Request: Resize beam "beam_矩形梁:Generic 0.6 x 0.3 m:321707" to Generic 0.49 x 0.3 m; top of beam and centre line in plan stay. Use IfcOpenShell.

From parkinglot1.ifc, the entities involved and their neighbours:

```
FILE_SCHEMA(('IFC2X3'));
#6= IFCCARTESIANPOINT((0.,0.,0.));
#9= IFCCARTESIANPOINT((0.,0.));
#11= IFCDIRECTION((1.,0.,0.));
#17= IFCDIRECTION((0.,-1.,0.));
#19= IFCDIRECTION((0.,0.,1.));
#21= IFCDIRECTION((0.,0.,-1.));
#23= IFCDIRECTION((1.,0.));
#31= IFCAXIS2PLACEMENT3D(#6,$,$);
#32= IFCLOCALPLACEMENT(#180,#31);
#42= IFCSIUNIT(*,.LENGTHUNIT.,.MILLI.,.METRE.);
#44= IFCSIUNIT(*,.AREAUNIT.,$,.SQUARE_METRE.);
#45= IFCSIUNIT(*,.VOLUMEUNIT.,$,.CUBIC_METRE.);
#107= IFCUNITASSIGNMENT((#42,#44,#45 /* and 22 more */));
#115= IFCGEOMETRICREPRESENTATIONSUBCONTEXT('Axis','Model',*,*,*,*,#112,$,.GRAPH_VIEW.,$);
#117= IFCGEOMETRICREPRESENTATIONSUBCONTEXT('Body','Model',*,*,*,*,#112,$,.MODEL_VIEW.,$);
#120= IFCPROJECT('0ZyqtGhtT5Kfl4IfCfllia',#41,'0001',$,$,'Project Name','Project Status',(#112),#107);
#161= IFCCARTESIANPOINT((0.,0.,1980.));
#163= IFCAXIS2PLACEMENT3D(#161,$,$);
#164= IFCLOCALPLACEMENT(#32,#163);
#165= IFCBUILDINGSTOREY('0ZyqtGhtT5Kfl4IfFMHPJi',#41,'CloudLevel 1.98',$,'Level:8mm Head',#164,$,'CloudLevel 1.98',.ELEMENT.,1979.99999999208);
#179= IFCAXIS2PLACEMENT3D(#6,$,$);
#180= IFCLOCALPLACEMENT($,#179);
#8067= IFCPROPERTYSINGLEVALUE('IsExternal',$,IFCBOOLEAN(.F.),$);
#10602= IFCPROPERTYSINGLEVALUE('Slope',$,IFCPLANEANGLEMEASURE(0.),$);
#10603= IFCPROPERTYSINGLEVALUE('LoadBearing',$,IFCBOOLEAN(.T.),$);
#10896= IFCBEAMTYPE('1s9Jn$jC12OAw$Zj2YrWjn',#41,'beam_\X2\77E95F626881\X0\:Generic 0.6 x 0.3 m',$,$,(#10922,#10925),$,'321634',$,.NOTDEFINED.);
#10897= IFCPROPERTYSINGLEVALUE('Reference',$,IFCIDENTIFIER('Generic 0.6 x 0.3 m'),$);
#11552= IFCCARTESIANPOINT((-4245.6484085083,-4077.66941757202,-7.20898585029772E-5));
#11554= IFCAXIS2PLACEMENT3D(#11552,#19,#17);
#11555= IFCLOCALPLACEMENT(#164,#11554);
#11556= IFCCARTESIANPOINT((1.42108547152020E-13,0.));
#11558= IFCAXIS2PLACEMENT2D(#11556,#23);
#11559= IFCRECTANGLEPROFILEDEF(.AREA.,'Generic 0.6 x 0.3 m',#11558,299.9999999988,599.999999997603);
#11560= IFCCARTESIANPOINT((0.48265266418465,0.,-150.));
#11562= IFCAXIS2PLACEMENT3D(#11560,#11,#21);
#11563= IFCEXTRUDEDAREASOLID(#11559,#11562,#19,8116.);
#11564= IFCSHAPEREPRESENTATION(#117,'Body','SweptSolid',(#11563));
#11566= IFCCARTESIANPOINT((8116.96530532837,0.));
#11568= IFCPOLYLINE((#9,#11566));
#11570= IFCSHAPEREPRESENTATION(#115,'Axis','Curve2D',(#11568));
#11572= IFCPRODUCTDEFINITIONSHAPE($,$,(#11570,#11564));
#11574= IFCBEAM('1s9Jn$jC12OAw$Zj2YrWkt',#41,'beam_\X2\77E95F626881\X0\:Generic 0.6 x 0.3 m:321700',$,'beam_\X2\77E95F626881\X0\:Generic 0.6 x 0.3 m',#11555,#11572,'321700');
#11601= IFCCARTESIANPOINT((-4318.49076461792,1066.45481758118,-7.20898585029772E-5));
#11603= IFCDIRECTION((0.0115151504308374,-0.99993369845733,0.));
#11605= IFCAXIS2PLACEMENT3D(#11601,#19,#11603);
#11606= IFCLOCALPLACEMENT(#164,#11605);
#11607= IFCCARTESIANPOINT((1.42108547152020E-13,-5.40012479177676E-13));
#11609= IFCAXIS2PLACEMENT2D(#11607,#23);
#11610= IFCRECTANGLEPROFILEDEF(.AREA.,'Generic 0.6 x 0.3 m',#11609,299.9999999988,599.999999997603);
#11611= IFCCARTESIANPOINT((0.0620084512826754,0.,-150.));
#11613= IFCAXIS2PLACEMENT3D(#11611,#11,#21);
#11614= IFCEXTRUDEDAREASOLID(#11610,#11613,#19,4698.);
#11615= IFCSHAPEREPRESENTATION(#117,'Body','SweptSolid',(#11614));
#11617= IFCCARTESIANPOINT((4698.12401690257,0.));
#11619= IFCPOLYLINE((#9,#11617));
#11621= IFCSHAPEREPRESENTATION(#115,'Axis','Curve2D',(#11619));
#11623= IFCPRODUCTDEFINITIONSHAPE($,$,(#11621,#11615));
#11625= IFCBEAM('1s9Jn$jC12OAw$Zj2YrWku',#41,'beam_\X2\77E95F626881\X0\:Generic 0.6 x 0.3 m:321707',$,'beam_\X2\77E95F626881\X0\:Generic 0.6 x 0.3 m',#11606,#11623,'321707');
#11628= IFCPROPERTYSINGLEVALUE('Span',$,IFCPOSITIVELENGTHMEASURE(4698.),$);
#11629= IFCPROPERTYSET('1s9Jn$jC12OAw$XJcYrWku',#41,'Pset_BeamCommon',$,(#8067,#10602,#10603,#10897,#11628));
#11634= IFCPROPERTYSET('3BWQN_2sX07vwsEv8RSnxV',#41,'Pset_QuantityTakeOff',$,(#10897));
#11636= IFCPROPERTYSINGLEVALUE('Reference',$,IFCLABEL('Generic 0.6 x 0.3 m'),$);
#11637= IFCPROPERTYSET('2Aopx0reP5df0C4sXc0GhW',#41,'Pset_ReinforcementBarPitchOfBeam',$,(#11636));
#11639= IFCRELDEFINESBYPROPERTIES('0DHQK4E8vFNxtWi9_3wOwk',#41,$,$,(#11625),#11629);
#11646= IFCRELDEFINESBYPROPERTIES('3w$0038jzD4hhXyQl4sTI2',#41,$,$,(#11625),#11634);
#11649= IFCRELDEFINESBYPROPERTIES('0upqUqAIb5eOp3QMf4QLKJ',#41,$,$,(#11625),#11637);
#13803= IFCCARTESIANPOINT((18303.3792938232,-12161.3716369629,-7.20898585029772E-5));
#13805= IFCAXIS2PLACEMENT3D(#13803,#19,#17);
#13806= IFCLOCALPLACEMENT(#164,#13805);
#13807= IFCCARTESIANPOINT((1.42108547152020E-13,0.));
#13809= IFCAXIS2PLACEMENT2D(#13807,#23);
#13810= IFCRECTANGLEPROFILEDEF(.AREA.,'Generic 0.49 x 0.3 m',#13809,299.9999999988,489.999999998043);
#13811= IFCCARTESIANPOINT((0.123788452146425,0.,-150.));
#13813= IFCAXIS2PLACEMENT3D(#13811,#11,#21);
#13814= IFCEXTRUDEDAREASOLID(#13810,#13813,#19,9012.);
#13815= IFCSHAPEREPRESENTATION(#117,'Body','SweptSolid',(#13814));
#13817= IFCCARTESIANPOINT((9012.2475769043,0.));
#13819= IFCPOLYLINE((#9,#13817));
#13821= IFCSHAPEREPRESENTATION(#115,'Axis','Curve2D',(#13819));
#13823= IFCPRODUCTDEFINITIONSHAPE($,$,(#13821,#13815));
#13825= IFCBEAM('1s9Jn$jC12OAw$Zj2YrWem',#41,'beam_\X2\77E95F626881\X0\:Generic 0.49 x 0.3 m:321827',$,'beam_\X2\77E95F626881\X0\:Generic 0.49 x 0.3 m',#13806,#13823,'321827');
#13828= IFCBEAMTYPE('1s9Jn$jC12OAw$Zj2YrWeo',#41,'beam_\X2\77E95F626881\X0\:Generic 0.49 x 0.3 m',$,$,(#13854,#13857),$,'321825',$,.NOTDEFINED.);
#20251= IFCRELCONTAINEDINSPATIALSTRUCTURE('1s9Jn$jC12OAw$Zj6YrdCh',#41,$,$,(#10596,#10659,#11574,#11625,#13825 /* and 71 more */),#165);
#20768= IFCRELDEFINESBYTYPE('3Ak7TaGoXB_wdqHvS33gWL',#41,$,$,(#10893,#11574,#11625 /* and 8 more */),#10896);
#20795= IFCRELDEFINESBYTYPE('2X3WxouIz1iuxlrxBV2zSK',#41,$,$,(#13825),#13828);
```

```python
import ifcopenshell
import ifcopenshell.api.pset
import ifcopenshell.api.type
import ifcopenshell.util.element
import ifcopenshell.util.representation

model = ifcopenshell.open("parkinglot1.ifc")

member = model.by_guid("1s9Jn$jC12OAw$Zj2YrWku")
source = next(p for p in model.by_type("IfcRectangleProfileDef") if p.ProfileName == "Generic 0.49 x 0.3 m")

body = ifcopenshell.util.representation.get_representation(member, "Model", "Body")
solid = body.Items[0]
old_profile = solid.SweptArea

# Copy the section's sizes but keep this member's own profile position.
profile = ifcopenshell.util.element.copy(model, source)
# Profiles are centred, so shift by half the change in depth to hold the top.
shift = (old_profile.XDim - profile.XDim) / 2
x, y = old_profile.Position.Location.Coordinates
up = (-1.0, 0.0)  # upwards, in the solid's own plane
location = model.createIfcCartesianPoint((x + up[0] * shift, y + up[1] * shift))
profile.Position = model.createIfcAxis2Placement2D(location, old_profile.Position.RefDirection)
solid.SweptArea = profile
if not model.get_total_inverses(old_profile):
    ifcopenshell.util.element.remove_deep2(model, old_profile)

new_type = model.by_guid("1s9Jn$jC12OAw$Zj2YrWeo")
ifcopenshell.api.type.assign_type(
    model, related_objects=[member], relating_type=new_type, should_map_representations=False
)
member.Name = member.Name.replace("Generic 0.6 x 0.3 m", "Generic 0.49 x 0.3 m")
member.ObjectType = "beam_矩形梁:Generic 0.49 x 0.3 m"
pset = model.by_id(ifcopenshell.util.element.get_pset(member, "Pset_BeamCommon", should_inherit=False)["id"])
ifcopenshell.api.pset.edit_pset(model, pset=pset, properties={"Reference": "Generic 0.49 x 0.3 m"})
pset = model.by_id(ifcopenshell.util.element.get_pset(member, "Pset_QuantityTakeOff", should_inherit=False)["id"])
ifcopenshell.api.pset.edit_pset(model, pset=pset, properties={"Reference": "Generic 0.49 x 0.3 m"})
pset = model.by_id(ifcopenshell.util.element.get_pset(member, "Pset_ReinforcementBarPitchOfBeam", should_inherit=False)["id"])
ifcopenshell.api.pset.edit_pset(model, pset=pset, properties={"Reference": "Generic 0.49 x 0.3 m"})

print(solid.SweptArea)

model.write("parkinglot1_rev.ifc")
```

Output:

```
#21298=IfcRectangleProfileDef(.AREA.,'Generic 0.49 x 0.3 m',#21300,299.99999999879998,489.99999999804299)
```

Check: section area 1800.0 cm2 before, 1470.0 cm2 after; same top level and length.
